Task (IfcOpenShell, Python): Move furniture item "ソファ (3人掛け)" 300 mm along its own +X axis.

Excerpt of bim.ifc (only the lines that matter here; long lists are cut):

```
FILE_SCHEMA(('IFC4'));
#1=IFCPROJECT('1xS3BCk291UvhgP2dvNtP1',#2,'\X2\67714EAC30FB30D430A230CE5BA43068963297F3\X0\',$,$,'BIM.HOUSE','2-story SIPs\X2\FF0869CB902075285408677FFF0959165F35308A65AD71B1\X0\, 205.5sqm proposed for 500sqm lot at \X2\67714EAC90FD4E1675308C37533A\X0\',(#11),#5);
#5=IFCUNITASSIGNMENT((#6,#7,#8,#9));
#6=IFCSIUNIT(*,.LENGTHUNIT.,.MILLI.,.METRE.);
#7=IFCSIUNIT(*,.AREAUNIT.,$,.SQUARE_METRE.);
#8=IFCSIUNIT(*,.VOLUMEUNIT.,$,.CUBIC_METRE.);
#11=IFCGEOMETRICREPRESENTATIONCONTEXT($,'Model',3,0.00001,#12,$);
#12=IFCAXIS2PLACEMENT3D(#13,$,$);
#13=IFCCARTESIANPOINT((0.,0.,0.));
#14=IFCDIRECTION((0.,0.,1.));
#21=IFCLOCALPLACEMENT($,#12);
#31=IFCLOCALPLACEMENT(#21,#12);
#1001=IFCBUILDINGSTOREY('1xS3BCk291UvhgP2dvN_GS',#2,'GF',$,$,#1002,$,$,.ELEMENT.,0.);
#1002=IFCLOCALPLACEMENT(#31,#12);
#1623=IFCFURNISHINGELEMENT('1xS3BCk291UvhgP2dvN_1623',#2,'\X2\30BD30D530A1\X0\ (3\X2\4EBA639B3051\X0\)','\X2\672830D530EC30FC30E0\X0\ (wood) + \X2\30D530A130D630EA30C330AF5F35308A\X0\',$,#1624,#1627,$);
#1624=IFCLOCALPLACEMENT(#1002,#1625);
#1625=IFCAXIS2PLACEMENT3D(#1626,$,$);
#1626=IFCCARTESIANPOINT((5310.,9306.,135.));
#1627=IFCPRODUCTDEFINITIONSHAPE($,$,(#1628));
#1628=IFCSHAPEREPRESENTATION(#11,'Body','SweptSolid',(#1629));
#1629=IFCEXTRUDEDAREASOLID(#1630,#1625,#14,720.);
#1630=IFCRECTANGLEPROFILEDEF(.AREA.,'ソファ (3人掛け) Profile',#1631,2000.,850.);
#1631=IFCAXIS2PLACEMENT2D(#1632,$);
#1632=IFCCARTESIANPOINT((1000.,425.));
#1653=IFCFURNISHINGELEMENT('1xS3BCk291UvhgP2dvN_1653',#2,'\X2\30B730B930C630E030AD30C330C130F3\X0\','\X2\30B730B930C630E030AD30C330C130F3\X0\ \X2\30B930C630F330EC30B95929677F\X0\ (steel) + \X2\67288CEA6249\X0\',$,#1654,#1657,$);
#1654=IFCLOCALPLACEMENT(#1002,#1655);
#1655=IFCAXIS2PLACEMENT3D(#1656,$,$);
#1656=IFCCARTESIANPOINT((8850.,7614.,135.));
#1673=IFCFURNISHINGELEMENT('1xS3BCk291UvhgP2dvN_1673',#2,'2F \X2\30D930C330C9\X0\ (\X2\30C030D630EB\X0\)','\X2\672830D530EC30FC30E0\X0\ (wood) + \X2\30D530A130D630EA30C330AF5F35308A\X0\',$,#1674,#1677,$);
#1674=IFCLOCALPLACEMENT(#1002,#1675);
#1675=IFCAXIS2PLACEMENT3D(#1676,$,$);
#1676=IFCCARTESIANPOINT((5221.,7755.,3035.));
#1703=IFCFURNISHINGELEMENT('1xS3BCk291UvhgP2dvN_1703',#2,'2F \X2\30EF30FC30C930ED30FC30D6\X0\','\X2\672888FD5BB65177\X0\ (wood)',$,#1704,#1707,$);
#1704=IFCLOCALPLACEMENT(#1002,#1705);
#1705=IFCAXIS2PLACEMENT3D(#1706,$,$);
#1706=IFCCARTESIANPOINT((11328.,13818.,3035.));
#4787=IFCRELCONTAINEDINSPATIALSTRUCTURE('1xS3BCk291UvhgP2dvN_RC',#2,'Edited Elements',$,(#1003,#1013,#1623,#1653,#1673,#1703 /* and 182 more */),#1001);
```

```python
import ifcopenshell
import ifcopenshell.api.geometry
import ifcopenshell.util.placement
import ifcopenshell.util.unit

model = ifcopenshell.open("bim.ifc")
unit_scale = ifcopenshell.util.unit.calculate_unit_scale(model)

item = model.by_guid("1xS3BCk291UvhgP2dvN_1623")
matrix = ifcopenshell.util.placement.get_local_placement(item.ObjectPlacement)
matrix[:3, 3] += matrix[:3, 0] * 0.3 / unit_scale
ifcopenshell.api.geometry.edit_object_placement(model, product=item, matrix=matrix, is_si=False)

print(ifcopenshell.util.placement.get_local_placement(item.ObjectPlacement).round(3) + 0.0)

model.write("bim_edited.ifc")
```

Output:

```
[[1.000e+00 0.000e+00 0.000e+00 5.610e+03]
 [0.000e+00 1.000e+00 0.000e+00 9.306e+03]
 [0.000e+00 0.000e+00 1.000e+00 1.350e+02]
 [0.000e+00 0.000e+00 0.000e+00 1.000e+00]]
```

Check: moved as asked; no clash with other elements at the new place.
